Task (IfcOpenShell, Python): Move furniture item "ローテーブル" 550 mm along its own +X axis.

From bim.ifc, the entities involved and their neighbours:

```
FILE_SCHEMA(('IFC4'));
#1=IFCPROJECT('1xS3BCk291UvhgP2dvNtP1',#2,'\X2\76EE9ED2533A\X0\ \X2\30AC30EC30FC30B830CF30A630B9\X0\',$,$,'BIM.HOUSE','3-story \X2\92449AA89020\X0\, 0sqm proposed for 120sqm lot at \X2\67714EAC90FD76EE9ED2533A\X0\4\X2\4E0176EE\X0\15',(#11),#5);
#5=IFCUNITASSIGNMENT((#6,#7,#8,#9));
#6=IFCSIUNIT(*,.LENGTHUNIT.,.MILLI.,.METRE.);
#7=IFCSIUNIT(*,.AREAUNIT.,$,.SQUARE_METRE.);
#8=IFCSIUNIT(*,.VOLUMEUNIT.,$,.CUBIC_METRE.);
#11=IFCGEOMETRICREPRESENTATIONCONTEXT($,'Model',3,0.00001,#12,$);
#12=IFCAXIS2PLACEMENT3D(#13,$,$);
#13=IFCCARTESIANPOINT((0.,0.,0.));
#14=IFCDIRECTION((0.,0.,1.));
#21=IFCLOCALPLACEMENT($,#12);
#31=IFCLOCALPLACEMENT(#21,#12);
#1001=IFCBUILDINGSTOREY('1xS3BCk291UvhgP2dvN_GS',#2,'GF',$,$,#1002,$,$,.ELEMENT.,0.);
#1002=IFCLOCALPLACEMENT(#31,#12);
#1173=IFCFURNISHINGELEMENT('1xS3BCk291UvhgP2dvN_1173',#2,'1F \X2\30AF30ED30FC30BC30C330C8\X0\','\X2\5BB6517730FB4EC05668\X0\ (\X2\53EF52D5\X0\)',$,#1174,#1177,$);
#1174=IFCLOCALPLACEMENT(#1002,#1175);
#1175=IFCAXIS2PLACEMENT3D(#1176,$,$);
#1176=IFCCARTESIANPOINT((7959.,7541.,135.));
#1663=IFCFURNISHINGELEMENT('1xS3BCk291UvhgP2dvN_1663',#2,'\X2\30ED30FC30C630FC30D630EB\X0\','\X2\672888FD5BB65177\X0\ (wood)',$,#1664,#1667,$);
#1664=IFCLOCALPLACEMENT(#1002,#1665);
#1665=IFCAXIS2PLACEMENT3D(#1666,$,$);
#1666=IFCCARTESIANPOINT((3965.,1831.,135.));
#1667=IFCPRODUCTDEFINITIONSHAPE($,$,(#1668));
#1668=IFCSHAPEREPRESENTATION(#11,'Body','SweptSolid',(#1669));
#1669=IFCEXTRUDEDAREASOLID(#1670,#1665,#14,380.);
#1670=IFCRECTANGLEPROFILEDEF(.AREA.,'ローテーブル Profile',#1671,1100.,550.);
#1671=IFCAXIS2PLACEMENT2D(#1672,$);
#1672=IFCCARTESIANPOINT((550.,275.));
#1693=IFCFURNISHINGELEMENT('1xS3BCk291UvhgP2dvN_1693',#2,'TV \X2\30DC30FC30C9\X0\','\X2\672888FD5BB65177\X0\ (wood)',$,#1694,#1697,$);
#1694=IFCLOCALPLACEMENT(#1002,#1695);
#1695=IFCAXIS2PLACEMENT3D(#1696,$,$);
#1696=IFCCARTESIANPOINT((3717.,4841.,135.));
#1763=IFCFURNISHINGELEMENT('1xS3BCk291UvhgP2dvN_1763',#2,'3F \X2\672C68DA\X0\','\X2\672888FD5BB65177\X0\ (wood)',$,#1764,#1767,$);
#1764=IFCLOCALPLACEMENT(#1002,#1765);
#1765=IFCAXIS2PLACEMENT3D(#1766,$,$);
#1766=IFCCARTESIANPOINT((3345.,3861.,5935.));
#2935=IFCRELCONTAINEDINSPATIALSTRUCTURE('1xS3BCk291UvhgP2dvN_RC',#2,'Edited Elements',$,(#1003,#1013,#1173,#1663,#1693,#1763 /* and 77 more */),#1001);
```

```python
import ifcopenshell
import ifcopenshell.api.geometry
import ifcopenshell.util.placement

model = ifcopenshell.open("bim.ifc")

item = model.by_guid("1xS3BCk291UvhgP2dvN_1663")
matrix = ifcopenshell.util.placement.get_local_placement(item.ObjectPlacement)
matrix[:3, 3] += matrix[:3, 0] * 550.0
ifcopenshell.api.geometry.edit_object_placement(model, product=item, matrix=matrix, is_si=False)

print(ifcopenshell.util.placement.get_local_placement(item.ObjectPlacement).round(3) + 0.0)

model.write("bim_rev.ifc")
```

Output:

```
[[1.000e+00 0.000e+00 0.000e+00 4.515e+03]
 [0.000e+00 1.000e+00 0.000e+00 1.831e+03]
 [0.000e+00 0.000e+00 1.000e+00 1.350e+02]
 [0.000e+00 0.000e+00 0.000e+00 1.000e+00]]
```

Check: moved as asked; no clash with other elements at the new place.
